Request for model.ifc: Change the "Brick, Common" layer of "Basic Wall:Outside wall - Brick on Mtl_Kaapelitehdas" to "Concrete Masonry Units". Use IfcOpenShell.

First a look at what the model holds.

```python
import ifcopenshell
import ifcopenshell.util.element

model = ifcopenshell.open("model.ifc")
print(model.schema)
for layer_set in model.by_type("IfcMaterialLayerSet"):
    if layer_set.LayerSetName == "Basic Wall:Outside wall - Brick on Mtl_Kaapelitehdas":
        for layer in layer_set.MaterialLayers:
            print(layer.id(), layer.Material and layer.Material.Name, layer.LayerThickness, sep=" | ")
        print(len(ifcopenshell.util.element.get_elements_by_material(model, layer_set)), "elements and types use it")
print(sorted(m.Name for m in model.by_type("IfcMaterial") if m.Name)[:60])
```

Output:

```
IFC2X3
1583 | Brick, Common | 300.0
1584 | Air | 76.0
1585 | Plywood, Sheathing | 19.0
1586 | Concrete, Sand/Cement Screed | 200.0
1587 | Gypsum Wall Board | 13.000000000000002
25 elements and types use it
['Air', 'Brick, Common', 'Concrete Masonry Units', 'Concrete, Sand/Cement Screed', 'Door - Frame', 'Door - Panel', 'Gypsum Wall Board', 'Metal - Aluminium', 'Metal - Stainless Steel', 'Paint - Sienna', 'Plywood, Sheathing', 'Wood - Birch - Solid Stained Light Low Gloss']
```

```python
import ifcopenshell
import ifcopenshell.api.material

model = ifcopenshell.open("model.ifc")

layer_set = next(s for s in model.by_type("IfcMaterialLayerSet") if s.LayerSetName == "Basic Wall:Outside wall - Brick on Mtl_Kaapelitehdas")
layer = next(l for l in layer_set.MaterialLayers if l.Material and l.Material.Name == "Brick, Common")
material = next(m for m in model.by_type("IfcMaterial") if m.Name == "Concrete Masonry Units")

# Point this one layer at the other material; renaming the old one would change it everywhere.
ifcopenshell.api.material.edit_layer(model, layer=layer, attributes={}, material=material)

print([l.Material.Name if l.Material else None for l in layer_set.MaterialLayers])

model.write("model_updated.ifc")
```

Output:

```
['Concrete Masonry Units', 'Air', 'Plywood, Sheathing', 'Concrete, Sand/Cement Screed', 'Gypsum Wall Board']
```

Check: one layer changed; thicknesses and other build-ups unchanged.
